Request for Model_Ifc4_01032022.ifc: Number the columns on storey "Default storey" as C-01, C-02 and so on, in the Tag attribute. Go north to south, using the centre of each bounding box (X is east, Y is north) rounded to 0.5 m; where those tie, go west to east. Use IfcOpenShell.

First a look at what the model holds.

```python
import ifcopenshell
import ifcopenshell.util.element
import ifcopenshell.util.placement

model = ifcopenshell.open("Model_Ifc4_01032022.ifc")
print(model.schema)
storey = next(s for s in model.by_type("IfcBuildingStorey") if s.Name == "Default storey")
columns = [e for e in ifcopenshell.util.element.get_decomposition(storey) if e.is_a("IfcColumn")]
for e in sorted(columns, key=lambda e: e.id()):
    origin = ifcopenshell.util.placement.get_local_placement(e.ObjectPlacement)[:3, 3]
    print(e.id(), e.Tag, e.Name, origin.round(2) + 0.0, sep=" | ")
```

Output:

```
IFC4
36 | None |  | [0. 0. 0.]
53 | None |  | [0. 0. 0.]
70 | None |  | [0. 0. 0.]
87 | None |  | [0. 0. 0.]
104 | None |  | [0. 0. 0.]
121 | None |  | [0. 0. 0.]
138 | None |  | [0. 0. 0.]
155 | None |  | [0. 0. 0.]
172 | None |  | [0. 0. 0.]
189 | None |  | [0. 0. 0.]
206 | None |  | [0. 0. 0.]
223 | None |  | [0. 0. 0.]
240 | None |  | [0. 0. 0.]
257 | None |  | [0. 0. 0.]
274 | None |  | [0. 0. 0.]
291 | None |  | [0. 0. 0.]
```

```python
import ifcopenshell
import ifcopenshell.geom
import ifcopenshell.util.element
import ifcopenshell.util.shape

model = ifcopenshell.open("Model_Ifc4_01032022.ifc")
settings = ifcopenshell.geom.settings()
settings.set("use-world-coords", True)


def centre(element):
    shape = ifcopenshell.geom.create_shape(settings, element)
    return ifcopenshell.util.shape.get_bbox_centroid(shape.geometry)


storey = next(s for s in model.by_type("IfcBuildingStorey") if s.Name == "Default storey")
columns = [e for e in ifcopenshell.util.element.get_decomposition(storey) if e.is_a("IfcColumn")]

# Insertion points can sit at a corner or the storey origin, so sort by the geometry (in metres).
centres = {e: centre(e) for e in columns}
columns.sort(key=lambda e: (-round(centres[e][1] / 0.5), centres[e][0]))

for i, e in enumerate(columns, start=1):
    number = f"C-{i:02d}"
    e.Tag = number
    print(e.id(), number)

model.write("Model_Ifc4_01032022_rev.ifc")
```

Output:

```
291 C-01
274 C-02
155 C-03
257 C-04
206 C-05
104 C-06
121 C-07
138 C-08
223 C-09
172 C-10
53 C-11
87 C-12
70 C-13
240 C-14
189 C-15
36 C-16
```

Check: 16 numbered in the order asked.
